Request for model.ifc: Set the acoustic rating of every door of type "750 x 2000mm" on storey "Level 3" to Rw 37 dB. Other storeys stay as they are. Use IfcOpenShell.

First a look at what the model holds.

```python
import ifcopenshell
import ifcopenshell.util.element

model = ifcopenshell.open("model.ifc")
print(model.schema)
storey = next(s for s in model.by_type("IfcBuildingStorey") if s.Name == "Level 3")
doors = [e for e in ifcopenshell.util.element.get_decomposition(storey) if e.is_a("IfcDoor")]
seen = {}
for e in doors:
    element_type = ifcopenshell.util.element.get_type(e)
    key = (element_type.Name if element_type != e and element_type else None, ifcopenshell.util.element.get_pset(e, "Pset_DoorCommon", "AcousticRating"))
    seen[key] = seen.get(key, 0) + 1
for (name, value), count in sorted(seen.items(), key=str):
    print(count, "x", name, "|", value)
```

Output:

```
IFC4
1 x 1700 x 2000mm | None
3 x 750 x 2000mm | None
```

```python
import ifcopenshell
import ifcopenshell.api.pset
import ifcopenshell.util.element

model = ifcopenshell.open("model.ifc")

storey = next(s for s in model.by_type("IfcBuildingStorey") if s.Name == "Level 3")
doors = [e for e in ifcopenshell.util.element.get_decomposition(storey) if e.is_a("IfcDoor")]

count = 0
for e in doors:
    element_type = ifcopenshell.util.element.get_type(e)
    if element_type in (None, e) or element_type.Name != "750 x 2000mm":
        continue
    # add_pset returns the element's existing set when there is one.
    pset = ifcopenshell.api.pset.add_pset(model, product=e, name="Pset_DoorCommon")
    ifcopenshell.api.pset.edit_pset(model, pset=pset, properties={"AcousticRating": "Rw 37 dB"})
    count += 1

print(count, "doors updated")

model.write("model_rev.ifc")
```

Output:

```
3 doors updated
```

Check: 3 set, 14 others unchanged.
